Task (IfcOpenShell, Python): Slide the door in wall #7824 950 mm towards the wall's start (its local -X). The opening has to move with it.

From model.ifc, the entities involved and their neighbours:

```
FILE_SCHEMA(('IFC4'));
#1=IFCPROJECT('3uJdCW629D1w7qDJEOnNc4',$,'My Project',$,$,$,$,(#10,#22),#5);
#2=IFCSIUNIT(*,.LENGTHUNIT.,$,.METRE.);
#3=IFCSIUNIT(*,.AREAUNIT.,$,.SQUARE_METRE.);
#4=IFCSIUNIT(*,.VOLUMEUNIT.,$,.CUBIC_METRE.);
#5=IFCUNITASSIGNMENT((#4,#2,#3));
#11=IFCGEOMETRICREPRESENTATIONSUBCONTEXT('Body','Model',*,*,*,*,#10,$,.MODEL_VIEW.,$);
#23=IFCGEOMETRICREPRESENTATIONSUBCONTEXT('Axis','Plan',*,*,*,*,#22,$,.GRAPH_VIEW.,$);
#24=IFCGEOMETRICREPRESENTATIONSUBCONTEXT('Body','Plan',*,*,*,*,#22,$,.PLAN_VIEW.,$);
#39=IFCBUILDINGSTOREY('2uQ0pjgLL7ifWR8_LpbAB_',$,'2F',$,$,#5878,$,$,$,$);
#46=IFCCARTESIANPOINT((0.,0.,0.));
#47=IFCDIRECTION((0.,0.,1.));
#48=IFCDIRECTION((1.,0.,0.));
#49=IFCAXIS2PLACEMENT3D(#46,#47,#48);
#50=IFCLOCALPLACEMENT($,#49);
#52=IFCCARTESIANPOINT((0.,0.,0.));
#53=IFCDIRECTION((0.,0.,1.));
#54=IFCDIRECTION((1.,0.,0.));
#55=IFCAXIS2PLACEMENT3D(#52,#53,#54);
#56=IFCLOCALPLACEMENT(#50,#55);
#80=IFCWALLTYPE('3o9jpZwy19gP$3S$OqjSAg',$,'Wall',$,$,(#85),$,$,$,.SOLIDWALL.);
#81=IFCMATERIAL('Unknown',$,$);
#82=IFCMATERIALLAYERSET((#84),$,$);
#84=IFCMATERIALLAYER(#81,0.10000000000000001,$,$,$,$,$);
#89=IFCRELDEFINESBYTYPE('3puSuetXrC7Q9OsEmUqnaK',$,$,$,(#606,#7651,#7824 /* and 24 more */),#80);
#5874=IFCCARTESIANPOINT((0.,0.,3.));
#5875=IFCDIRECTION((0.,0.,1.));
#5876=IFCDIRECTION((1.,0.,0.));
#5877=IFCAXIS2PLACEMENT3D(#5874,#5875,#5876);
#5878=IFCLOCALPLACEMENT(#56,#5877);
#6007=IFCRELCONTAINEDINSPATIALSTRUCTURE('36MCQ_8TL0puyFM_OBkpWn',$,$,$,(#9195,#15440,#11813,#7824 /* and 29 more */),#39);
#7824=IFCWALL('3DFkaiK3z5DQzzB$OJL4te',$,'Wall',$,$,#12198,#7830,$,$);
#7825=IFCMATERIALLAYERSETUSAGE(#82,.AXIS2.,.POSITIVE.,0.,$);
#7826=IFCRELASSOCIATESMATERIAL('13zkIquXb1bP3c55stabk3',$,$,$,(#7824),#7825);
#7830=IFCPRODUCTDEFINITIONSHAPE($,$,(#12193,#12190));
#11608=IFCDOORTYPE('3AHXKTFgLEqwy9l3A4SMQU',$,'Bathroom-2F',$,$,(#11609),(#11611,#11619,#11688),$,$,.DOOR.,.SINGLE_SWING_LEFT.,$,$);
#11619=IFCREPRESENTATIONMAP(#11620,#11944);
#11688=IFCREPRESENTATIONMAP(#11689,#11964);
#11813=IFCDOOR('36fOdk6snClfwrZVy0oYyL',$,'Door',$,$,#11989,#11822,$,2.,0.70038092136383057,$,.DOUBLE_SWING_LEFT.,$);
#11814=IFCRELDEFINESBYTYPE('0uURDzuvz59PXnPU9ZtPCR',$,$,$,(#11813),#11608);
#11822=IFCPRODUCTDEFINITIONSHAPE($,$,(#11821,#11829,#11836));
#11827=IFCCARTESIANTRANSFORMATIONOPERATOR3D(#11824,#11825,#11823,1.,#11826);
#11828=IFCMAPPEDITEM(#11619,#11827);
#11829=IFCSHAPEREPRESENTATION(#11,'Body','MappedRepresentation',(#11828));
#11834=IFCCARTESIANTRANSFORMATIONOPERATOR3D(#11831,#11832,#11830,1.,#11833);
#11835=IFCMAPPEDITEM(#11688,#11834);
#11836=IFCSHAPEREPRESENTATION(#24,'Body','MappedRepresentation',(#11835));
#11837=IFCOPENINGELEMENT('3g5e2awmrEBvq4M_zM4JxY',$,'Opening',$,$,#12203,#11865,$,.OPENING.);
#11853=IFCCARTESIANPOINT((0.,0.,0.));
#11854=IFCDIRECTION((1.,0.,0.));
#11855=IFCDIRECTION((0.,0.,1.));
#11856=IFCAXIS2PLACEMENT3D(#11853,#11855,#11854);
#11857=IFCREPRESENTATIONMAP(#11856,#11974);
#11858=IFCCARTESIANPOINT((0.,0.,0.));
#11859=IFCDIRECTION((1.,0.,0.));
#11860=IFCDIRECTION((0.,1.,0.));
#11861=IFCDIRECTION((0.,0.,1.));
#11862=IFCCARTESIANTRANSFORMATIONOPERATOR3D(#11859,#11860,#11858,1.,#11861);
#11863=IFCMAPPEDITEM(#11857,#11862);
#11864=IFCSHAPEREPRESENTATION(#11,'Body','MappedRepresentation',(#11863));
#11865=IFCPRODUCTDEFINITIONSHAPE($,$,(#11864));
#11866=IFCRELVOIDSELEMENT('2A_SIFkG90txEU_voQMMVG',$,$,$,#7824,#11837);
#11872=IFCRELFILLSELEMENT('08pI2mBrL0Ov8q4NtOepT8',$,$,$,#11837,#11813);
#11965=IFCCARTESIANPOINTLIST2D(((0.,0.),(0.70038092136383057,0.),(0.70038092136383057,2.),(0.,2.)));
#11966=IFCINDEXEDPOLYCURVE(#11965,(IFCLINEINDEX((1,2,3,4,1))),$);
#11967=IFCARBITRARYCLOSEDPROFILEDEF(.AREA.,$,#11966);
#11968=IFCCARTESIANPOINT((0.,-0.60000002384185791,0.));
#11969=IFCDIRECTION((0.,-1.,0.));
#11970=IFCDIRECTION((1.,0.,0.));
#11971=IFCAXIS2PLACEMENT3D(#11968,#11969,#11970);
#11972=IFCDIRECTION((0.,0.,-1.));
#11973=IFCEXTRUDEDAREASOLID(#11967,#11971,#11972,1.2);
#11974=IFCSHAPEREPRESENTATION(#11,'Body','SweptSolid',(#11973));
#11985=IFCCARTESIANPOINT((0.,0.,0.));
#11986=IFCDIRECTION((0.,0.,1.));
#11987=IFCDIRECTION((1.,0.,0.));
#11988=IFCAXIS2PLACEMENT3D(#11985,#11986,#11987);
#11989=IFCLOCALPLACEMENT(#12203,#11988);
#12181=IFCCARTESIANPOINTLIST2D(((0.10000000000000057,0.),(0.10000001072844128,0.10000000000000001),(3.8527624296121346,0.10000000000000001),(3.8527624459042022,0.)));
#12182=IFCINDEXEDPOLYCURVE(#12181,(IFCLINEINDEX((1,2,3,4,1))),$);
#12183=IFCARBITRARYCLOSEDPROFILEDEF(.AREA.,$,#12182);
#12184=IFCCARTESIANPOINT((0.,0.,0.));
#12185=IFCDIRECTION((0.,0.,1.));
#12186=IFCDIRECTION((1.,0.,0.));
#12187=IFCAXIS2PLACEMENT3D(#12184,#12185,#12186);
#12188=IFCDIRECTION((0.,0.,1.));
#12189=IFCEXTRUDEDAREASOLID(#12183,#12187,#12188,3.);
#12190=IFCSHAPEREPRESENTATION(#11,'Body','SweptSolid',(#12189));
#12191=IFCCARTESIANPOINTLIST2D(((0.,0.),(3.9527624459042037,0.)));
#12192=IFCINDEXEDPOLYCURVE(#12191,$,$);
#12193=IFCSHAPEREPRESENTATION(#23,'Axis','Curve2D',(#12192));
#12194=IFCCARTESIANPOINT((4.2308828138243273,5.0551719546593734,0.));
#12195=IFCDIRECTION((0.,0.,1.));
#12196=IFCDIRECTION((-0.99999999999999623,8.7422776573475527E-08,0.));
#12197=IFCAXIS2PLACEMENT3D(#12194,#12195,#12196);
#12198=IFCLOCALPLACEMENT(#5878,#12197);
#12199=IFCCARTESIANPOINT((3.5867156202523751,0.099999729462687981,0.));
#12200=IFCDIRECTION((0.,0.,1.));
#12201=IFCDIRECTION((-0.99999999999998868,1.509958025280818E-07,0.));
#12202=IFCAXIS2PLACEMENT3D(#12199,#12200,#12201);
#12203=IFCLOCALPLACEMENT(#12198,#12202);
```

```python
import ifcopenshell
import ifcopenshell.api.geometry
import ifcopenshell.util.placement
import ifcopenshell.util.unit

model = ifcopenshell.open("model.ifc")
unit_scale = ifcopenshell.util.unit.calculate_unit_scale(model)

door = model.by_id(11813)
opening = door.FillsVoids[0].RelatingOpeningElement
wall = opening.VoidsElements[0].RelatingBuildingElement

wall_matrix = ifcopenshell.util.placement.get_local_placement(wall.ObjectPlacement)
shift = wall_matrix[:3, 0] * -0.95 / unit_scale
before = ifcopenshell.util.placement.get_local_placement(door.ObjectPlacement)[:3, 3].copy()

# The door is placed relative to its opening, so it follows when the opening moves.
matrix = ifcopenshell.util.placement.get_local_placement(opening.ObjectPlacement)
matrix[:3, 3] += shift
ifcopenshell.api.geometry.edit_object_placement(
    model, product=opening, matrix=matrix, is_si=False, should_transform_children=True
)

after = ifcopenshell.util.placement.get_local_placement(door.ObjectPlacement)[:3, 3]
print("door moved by", (after - before).round(3) + 0.0)

model.write("model_updated.ifc")
```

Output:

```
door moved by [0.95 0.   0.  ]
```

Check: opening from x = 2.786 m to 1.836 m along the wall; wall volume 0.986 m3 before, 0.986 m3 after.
